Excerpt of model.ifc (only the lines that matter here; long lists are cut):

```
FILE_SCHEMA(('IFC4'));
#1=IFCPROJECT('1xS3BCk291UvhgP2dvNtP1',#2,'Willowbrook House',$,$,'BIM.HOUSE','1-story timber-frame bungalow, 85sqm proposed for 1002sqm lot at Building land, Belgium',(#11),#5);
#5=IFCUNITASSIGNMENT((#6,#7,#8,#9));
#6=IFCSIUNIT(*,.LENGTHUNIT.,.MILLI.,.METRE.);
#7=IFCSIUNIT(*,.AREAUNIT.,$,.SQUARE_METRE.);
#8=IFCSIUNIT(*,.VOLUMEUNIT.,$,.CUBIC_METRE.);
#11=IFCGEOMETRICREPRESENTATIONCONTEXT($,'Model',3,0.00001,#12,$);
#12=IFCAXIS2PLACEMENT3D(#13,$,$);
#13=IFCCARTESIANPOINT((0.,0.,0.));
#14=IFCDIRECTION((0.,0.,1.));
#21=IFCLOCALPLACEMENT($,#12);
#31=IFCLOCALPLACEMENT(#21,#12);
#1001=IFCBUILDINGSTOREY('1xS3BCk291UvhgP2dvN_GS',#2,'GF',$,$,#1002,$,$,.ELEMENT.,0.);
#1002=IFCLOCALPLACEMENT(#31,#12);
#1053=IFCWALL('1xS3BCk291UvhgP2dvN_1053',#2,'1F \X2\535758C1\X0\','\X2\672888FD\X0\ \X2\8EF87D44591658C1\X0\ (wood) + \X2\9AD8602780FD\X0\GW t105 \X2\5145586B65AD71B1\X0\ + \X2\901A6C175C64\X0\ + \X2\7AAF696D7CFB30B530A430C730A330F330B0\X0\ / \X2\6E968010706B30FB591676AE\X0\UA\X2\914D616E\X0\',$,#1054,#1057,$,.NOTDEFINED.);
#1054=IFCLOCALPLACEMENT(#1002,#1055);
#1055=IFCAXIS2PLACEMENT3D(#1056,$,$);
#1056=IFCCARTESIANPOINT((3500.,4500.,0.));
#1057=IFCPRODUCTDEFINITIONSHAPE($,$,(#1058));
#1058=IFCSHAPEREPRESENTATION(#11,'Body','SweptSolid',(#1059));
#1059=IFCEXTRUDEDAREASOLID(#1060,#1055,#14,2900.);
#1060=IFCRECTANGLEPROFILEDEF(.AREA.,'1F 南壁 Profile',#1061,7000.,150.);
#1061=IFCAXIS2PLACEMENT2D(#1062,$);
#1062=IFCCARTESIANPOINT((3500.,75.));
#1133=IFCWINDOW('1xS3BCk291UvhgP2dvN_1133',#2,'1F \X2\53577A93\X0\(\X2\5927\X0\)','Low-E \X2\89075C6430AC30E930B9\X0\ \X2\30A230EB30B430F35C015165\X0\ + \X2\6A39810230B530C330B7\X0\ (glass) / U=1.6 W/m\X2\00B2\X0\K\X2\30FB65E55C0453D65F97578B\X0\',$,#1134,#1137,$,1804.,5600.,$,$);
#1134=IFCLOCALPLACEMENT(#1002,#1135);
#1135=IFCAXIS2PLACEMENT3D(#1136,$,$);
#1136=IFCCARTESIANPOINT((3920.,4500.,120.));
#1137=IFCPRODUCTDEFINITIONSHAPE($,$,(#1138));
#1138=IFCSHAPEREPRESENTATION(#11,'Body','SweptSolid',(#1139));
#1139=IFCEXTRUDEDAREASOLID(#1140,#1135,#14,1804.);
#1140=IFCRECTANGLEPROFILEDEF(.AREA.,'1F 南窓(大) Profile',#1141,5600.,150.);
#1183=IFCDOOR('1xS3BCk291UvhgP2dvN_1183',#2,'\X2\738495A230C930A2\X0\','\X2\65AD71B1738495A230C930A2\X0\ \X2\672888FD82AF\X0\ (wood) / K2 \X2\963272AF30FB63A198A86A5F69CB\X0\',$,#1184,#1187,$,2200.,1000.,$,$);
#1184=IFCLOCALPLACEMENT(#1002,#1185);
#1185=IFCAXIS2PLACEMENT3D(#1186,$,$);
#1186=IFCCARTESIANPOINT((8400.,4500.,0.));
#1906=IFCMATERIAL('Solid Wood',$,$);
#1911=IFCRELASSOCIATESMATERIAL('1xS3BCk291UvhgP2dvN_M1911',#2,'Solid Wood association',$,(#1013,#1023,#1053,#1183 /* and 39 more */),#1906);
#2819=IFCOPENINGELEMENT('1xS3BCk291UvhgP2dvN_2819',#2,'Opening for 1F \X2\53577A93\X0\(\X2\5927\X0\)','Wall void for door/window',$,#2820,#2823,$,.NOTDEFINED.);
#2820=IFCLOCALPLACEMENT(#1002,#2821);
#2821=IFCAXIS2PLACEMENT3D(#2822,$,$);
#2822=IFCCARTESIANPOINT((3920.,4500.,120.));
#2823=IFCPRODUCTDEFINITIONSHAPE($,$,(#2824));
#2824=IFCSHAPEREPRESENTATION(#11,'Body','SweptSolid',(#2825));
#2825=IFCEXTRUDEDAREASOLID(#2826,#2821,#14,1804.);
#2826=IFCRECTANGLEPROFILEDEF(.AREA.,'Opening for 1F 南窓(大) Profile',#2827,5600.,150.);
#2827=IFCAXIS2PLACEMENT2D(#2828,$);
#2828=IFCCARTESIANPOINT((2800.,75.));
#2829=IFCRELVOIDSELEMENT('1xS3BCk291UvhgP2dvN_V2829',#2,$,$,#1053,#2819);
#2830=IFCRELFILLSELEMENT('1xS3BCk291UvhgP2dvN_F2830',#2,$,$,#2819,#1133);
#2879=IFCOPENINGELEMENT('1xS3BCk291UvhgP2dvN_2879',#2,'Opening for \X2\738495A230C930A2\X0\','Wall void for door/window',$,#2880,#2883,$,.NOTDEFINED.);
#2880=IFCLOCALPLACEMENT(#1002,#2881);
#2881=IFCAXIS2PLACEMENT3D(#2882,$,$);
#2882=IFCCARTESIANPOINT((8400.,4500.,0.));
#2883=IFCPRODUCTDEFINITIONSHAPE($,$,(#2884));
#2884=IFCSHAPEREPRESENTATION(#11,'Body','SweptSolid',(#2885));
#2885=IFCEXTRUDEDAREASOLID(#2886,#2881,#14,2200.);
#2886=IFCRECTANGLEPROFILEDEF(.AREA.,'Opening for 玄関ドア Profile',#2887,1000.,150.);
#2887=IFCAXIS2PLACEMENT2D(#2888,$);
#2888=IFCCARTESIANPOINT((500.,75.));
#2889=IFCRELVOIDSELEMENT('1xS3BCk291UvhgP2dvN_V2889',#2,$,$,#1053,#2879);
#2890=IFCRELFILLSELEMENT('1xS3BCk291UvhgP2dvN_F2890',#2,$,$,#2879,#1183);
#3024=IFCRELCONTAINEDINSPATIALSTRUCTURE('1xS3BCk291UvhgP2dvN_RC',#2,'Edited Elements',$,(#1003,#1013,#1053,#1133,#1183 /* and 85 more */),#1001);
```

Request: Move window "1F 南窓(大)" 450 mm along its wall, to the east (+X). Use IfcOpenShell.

```python
import ifcopenshell
import ifcopenshell.api.geometry
import ifcopenshell.util.placement
import ifcopenshell.util.unit

model = ifcopenshell.open("model.ifc")
unit_scale = ifcopenshell.util.unit.calculate_unit_scale(model)

window = model.by_guid("1xS3BCk291UvhgP2dvN_1133")
opening = window.FillsVoids[0].RelatingOpeningElement
wall = opening.VoidsElements[0].RelatingBuildingElement

wall_matrix = ifcopenshell.util.placement.get_local_placement(wall.ObjectPlacement)
shift = wall_matrix[:3, 0] * 0.45 / unit_scale
before = ifcopenshell.util.placement.get_local_placement(window.ObjectPlacement)[:3, 3].copy()

# The window is not placed relative to its opening, so move both.
for product in (opening, window):
    matrix = ifcopenshell.util.placement.get_local_placement(product.ObjectPlacement)
    matrix[:3, 3] += shift
    ifcopenshell.api.geometry.edit_object_placement(model, product=product, matrix=matrix, is_si=False)

after = ifcopenshell.util.placement.get_local_placement(window.ObjectPlacement)[:3, 3]
print("window moved by", (after - before).round(3) + 0.0)

model.write("model_rev.ifc")
```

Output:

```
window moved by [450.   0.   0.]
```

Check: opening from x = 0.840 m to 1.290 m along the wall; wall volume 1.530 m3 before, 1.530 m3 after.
